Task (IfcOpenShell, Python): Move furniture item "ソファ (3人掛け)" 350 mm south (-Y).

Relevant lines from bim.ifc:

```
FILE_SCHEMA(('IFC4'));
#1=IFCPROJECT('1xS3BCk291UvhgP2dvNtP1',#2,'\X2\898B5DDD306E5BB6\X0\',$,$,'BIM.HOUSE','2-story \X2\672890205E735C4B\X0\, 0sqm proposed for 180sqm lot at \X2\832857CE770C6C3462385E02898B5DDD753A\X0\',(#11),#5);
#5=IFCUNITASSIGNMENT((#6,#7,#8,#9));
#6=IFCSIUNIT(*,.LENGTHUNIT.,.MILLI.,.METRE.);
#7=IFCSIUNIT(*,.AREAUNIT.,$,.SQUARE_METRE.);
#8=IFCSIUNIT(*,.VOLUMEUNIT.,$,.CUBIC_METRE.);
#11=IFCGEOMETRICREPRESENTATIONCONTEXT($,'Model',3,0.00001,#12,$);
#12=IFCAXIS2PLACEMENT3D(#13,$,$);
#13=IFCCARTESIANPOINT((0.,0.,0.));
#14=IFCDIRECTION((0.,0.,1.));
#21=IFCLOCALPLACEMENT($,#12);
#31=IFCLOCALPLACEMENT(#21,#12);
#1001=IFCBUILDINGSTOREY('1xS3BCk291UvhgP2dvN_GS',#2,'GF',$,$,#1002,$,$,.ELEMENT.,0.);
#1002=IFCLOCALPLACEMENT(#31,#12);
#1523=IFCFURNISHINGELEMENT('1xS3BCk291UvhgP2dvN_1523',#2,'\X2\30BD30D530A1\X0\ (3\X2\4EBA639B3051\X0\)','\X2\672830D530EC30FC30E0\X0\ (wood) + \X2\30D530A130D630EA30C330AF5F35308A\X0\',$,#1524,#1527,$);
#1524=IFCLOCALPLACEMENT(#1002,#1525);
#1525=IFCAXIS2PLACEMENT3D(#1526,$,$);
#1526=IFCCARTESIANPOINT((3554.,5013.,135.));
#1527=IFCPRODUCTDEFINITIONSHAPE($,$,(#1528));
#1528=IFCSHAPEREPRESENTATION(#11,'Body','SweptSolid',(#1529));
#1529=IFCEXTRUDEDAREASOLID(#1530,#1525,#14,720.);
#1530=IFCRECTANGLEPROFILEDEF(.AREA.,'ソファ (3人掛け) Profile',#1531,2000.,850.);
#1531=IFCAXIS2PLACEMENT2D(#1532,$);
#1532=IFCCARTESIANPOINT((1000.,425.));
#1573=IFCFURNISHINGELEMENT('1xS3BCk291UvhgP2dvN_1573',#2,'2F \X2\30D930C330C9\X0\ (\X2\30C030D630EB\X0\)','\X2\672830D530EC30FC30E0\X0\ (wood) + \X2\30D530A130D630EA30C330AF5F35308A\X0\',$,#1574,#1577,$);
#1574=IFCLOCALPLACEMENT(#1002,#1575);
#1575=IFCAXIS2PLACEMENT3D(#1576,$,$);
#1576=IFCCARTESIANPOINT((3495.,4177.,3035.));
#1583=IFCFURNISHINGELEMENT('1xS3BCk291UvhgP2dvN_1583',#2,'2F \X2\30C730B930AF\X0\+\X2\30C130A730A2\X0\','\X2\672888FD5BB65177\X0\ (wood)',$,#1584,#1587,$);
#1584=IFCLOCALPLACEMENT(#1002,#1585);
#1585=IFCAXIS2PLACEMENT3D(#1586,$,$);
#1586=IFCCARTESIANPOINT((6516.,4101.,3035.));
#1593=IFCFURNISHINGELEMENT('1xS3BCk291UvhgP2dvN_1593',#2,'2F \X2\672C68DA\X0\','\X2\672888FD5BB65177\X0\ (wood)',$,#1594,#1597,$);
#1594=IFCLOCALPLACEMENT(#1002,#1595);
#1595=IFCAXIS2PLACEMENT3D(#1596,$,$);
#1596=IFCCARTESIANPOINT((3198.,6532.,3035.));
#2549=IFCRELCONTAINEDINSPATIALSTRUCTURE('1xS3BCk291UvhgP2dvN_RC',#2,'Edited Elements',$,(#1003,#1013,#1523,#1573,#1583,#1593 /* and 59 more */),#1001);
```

```python
import ifcopenshell
import ifcopenshell.api.geometry
import ifcopenshell.util.placement
import ifcopenshell.util.unit

model = ifcopenshell.open("bim.ifc")
unit_scale = ifcopenshell.util.unit.calculate_unit_scale(model)

item = model.by_id(1523)
matrix = ifcopenshell.util.placement.get_local_placement(item.ObjectPlacement)
matrix[1, 3] -= 0.35 / unit_scale
ifcopenshell.api.geometry.edit_object_placement(model, product=item, matrix=matrix, is_si=False)

print(ifcopenshell.util.placement.get_local_placement(item.ObjectPlacement).round(3) + 0.0)

model.write("bim_rev.ifc")
```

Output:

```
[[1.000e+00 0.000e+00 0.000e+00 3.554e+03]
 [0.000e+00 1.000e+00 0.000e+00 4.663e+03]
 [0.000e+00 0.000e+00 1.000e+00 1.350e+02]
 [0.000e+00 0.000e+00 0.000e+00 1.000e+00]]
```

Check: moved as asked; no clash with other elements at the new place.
